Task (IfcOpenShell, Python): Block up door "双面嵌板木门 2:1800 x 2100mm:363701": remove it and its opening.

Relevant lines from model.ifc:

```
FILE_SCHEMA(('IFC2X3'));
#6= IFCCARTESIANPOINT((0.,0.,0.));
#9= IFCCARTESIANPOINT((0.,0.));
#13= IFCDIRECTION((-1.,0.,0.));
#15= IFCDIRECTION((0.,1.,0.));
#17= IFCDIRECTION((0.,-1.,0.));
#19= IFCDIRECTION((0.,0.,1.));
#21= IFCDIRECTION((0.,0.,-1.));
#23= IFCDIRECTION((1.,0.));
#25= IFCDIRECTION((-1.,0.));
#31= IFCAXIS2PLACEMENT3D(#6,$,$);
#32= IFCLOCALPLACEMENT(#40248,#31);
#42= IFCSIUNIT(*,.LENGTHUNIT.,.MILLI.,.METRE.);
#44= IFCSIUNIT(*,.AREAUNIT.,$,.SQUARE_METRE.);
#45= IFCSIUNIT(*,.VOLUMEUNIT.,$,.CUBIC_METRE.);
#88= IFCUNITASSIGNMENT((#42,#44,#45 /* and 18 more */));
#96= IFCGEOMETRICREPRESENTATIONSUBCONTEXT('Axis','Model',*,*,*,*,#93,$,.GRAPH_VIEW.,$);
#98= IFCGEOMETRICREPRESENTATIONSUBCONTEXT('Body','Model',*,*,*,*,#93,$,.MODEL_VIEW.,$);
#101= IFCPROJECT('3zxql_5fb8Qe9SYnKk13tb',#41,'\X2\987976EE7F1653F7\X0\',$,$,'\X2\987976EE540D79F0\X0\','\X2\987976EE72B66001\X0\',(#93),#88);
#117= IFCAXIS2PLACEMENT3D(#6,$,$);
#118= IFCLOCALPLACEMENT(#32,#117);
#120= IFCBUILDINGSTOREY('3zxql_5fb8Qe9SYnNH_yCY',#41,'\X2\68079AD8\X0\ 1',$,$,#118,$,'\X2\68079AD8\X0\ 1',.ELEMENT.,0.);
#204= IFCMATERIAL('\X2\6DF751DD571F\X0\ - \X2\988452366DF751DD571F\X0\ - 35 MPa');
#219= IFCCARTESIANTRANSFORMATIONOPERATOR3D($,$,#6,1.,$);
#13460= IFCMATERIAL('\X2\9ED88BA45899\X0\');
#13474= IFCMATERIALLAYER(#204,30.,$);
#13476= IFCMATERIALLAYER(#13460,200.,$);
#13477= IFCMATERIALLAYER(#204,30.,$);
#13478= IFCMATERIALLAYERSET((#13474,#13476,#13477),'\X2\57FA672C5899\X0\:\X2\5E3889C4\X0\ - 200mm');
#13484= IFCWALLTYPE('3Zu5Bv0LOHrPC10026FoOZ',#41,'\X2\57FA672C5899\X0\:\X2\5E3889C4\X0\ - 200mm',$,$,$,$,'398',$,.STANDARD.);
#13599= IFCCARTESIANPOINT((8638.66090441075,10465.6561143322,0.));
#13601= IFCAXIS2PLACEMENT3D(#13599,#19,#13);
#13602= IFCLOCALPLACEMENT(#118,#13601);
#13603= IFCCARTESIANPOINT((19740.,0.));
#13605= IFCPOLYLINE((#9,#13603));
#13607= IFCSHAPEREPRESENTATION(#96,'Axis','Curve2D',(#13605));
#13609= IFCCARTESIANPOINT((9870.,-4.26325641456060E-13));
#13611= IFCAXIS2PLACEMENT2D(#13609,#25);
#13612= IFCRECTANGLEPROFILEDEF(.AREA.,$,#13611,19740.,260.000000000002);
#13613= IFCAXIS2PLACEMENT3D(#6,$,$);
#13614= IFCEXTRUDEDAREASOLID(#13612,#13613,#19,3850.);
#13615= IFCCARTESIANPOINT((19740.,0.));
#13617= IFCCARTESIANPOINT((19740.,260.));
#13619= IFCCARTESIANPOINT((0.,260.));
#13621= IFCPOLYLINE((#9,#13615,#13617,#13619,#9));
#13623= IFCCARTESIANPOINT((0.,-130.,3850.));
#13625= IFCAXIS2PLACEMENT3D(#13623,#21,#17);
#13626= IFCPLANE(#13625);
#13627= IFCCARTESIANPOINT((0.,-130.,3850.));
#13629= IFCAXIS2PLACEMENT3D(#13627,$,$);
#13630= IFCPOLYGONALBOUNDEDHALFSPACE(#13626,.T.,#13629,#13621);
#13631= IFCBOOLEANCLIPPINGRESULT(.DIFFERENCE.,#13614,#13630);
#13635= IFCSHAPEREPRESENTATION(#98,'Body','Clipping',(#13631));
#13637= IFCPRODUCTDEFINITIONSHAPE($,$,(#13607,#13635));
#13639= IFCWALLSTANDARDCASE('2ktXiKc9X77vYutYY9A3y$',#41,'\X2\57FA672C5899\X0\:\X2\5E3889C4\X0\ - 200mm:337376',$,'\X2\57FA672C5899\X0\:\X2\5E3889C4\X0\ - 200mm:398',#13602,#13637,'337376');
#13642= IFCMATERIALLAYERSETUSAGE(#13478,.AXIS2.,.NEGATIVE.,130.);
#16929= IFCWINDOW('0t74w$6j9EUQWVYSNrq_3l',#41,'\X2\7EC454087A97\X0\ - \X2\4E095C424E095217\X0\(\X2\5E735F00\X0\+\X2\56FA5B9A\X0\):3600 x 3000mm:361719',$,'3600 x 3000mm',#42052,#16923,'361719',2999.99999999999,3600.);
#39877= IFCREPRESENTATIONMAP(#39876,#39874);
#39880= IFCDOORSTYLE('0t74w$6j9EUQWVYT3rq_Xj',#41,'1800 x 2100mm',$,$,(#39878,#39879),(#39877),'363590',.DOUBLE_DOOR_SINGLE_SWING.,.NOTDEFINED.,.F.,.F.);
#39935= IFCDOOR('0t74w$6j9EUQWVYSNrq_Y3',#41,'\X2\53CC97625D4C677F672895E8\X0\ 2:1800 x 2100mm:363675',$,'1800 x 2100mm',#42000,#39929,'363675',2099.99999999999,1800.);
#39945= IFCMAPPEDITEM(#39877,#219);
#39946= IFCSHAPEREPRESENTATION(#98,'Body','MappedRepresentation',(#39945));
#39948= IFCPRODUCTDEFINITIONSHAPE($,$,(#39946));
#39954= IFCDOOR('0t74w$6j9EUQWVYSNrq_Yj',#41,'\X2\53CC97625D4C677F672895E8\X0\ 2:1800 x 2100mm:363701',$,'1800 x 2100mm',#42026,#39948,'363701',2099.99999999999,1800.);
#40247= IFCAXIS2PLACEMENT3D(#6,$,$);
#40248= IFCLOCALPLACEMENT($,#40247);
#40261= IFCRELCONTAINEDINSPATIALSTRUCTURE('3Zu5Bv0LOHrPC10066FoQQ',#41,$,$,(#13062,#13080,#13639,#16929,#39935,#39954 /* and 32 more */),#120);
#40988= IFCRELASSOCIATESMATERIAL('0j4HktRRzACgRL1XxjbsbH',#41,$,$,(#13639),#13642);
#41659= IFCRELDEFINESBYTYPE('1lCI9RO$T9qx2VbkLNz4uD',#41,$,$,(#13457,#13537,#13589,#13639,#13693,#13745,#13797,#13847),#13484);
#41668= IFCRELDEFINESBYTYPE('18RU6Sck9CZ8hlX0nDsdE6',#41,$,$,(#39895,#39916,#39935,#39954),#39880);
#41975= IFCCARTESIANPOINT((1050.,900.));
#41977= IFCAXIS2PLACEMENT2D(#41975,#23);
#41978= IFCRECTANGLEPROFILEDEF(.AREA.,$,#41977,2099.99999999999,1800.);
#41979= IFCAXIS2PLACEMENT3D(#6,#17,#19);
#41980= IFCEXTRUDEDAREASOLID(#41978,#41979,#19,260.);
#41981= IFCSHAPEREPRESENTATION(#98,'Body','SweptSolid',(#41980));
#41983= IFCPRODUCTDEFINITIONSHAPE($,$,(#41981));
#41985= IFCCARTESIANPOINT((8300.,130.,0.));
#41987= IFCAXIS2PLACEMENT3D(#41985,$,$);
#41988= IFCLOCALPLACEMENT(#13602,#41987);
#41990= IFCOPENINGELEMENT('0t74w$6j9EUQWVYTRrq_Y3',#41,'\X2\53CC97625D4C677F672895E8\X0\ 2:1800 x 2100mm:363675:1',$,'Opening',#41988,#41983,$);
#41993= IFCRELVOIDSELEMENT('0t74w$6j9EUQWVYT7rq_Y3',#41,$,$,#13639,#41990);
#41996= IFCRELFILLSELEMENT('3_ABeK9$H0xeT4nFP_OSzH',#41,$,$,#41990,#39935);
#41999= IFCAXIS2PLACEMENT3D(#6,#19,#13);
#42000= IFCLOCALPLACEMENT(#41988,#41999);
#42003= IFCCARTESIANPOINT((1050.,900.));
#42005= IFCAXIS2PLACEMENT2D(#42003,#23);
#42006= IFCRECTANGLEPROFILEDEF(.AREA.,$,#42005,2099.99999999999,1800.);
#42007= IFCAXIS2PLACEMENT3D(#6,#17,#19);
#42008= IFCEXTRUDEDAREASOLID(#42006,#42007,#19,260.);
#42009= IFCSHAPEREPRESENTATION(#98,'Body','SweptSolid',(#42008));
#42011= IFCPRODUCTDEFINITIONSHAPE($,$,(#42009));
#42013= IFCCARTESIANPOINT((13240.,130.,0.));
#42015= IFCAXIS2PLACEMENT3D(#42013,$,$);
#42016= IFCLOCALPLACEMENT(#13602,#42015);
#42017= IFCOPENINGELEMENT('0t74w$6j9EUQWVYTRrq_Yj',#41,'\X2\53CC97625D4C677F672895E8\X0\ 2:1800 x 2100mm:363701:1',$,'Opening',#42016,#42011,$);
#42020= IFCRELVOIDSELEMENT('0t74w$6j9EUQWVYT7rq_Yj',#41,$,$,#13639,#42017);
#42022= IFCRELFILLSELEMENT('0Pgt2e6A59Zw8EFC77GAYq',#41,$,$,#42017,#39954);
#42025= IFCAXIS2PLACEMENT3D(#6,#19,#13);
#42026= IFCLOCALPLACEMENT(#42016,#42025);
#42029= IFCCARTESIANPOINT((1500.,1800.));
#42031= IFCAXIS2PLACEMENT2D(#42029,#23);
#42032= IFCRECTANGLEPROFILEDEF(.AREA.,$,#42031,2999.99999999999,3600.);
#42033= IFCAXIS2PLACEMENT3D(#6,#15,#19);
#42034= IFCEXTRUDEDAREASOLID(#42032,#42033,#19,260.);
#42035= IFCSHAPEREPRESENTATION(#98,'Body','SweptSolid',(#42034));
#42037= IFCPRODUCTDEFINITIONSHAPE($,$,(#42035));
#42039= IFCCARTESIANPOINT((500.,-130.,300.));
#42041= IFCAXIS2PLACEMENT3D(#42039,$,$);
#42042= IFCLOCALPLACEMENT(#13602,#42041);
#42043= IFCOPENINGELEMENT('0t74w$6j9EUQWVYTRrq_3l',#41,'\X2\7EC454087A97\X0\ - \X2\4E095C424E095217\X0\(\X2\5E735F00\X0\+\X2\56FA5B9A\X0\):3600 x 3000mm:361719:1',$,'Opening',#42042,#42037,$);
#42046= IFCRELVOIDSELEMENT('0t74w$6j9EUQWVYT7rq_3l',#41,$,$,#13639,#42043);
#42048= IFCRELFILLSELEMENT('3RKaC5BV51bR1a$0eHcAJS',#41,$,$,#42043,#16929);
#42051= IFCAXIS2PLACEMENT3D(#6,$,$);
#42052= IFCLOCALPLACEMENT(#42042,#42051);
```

```python
import ifcopenshell
import ifcopenshell.api.feature
import ifcopenshell.api.root
import ifcopenshell.geom
import ifcopenshell.util.shape

model = ifcopenshell.open("model.ifc")
settings = ifcopenshell.geom.settings()


def volume(element):
    """Net volume in cubic metres, openings subtracted."""
    shape = ifcopenshell.geom.create_shape(settings, element)
    return ifcopenshell.util.shape.get_volume(shape.geometry)


door = model.by_guid("0t74w$6j9EUQWVYSNrq_Yj")
opening = door.FillsVoids[0].RelatingOpeningElement
wall = opening.VoidsElements[0].RelatingBuildingElement
before = volume(wall)

ifcopenshell.api.root.remove_product(model, product=door)
ifcopenshell.api.feature.remove_feature(model, feature=opening)

after = volume(wall)

print(f"wall volume {before:.3f} -> {after:.3f} m3")

model.write("model_updated.ifc")
```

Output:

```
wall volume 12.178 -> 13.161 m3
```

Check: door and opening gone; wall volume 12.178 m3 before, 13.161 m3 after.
